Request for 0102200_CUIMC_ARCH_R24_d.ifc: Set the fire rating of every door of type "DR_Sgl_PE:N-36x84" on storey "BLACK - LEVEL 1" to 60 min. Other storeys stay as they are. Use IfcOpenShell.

First a look at what the model holds.

```python
import ifcopenshell
import ifcopenshell.util.element

model = ifcopenshell.open("0102200_CUIMC_ARCH_R24_d.ifc")
print(model.schema)
storey = next(s for s in model.by_type("IfcBuildingStorey") if s.Name == "BLACK - LEVEL 1")
doors = [e for e in ifcopenshell.util.element.get_decomposition(storey) if e.is_a("IfcDoor")]
seen = {}
for e in doors:
    element_type = ifcopenshell.util.element.get_type(e)
    key = (element_type.Name if element_type != e and element_type else None, ifcopenshell.util.element.get_pset(e, "Pset_DoorCommon", "FireRating"))
    seen[key] = seen.get(key, 0) + 1
for (name, value), count in sorted(seen.items(), key=str):
    print(count, "x", name, "|", value)
```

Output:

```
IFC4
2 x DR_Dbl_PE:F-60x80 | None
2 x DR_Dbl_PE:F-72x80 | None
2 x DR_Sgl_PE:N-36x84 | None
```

```python
import ifcopenshell
import ifcopenshell.api.pset
import ifcopenshell.util.element

model = ifcopenshell.open("0102200_CUIMC_ARCH_R24_d.ifc")

storey = next(s for s in model.by_type("IfcBuildingStorey") if s.Name == "BLACK - LEVEL 1")
doors = [e for e in ifcopenshell.util.element.get_decomposition(storey) if e.is_a("IfcDoor")]

count = 0
for e in doors:
    element_type = ifcopenshell.util.element.get_type(e)
    if element_type in (None, e) or element_type.Name != "DR_Sgl_PE:N-36x84":
        continue
    # add_pset returns the element's existing set when there is one.
    pset = ifcopenshell.api.pset.add_pset(model, product=e, name="Pset_DoorCommon")
    ifcopenshell.api.pset.edit_pset(model, pset=pset, properties={"FireRating": "60 min"})
    count += 1

print(count, "doors updated")

model.write("0102200_CUIMC_ARCH_R24_d_edited.ifc")
```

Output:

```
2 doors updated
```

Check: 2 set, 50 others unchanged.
